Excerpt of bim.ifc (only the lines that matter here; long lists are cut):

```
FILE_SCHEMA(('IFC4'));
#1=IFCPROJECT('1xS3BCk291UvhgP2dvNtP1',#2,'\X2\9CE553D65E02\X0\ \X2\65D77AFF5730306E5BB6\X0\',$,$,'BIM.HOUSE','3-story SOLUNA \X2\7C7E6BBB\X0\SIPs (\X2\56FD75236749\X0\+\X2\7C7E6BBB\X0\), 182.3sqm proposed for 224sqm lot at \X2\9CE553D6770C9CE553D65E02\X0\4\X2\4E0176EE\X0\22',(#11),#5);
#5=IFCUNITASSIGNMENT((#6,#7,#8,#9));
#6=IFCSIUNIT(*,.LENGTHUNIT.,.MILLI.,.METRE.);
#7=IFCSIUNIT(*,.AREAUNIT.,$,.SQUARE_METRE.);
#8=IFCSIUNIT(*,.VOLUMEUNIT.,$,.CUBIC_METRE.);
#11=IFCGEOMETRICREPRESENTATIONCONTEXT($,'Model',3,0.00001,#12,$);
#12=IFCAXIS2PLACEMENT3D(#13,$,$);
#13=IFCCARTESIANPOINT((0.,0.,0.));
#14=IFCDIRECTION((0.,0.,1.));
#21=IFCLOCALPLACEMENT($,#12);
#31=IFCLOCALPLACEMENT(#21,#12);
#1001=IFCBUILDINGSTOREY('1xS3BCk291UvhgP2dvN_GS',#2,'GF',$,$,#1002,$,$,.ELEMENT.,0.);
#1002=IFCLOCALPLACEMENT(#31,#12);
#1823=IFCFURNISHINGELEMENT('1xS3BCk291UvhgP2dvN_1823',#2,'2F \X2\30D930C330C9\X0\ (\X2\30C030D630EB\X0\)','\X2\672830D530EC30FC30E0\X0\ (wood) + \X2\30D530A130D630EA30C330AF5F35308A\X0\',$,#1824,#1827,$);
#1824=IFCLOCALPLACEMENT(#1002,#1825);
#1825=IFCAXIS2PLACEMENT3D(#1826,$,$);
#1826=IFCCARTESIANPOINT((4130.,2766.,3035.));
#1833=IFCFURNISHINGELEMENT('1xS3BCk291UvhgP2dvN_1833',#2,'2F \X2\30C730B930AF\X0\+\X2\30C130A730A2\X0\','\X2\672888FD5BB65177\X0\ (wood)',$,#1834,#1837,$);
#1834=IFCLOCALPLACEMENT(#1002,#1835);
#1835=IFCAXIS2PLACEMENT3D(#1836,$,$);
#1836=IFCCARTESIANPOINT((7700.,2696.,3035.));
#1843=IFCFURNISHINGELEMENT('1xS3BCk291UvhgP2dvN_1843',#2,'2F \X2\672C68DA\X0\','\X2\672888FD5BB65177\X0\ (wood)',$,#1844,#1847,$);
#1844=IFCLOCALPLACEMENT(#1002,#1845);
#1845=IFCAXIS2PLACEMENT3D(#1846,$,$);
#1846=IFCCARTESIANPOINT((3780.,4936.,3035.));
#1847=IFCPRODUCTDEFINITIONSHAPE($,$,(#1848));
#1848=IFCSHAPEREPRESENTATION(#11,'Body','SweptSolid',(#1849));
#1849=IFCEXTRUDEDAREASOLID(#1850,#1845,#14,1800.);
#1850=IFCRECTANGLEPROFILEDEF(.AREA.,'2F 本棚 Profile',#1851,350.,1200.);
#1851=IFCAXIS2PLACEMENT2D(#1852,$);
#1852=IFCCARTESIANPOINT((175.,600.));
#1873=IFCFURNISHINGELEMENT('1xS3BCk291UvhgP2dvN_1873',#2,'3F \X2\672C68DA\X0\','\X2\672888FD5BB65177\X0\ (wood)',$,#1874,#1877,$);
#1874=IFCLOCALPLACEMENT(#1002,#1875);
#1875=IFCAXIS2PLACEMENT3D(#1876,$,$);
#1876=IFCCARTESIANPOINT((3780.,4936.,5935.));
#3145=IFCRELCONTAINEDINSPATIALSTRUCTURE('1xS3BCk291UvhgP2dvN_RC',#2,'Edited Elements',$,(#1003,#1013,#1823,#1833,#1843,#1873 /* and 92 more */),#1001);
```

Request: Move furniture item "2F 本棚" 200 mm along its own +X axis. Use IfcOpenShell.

```python
import ifcopenshell
import ifcopenshell.api.geometry
import ifcopenshell.util.placement

model = ifcopenshell.open("bim.ifc")

item = model.by_guid("1xS3BCk291UvhgP2dvN_1843")
matrix = ifcopenshell.util.placement.get_local_placement(item.ObjectPlacement)
matrix[:3, 3] += matrix[:3, 0] * 200.0
ifcopenshell.api.geometry.edit_object_placement(model, product=item, matrix=matrix, is_si=False)

print(ifcopenshell.util.placement.get_local_placement(item.ObjectPlacement).round(3) + 0.0)

model.write("bim_edited.ifc")
```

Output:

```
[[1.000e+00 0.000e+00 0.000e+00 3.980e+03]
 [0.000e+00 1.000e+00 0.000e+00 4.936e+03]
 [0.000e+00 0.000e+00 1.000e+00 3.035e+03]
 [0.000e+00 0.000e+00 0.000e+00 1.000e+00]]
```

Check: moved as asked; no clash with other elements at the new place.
